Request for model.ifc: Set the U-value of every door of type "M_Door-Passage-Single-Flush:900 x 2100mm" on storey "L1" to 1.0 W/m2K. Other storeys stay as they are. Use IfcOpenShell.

First a look at what the model holds.

```python
import ifcopenshell
import ifcopenshell.util.element

model = ifcopenshell.open("model.ifc")
print(model.schema)
storey = next(s for s in model.by_type("IfcBuildingStorey") if s.Name == "L1")
doors = [e for e in ifcopenshell.util.element.get_decomposition(storey) if e.is_a("IfcDoor")]
seen = {}
for e in doors:
    element_type = ifcopenshell.util.element.get_type(e)
    key = (element_type.Name if element_type != e and element_type else None, ifcopenshell.util.element.get_pset(e, "Pset_DoorCommon", "ThermalTransmittance"))
    seen[key] = seen.get(key, 0) + 1
for (name, value), count in sorted(seen.items(), key=str):
    print(count, "x", name, "|", value)
```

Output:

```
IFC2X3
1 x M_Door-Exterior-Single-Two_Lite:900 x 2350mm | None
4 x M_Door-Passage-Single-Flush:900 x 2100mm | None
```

```python
import ifcopenshell
import ifcopenshell.api.pset
import ifcopenshell.util.element

model = ifcopenshell.open("model.ifc")

storey = next(s for s in model.by_type("IfcBuildingStorey") if s.Name == "L1")
doors = [e for e in ifcopenshell.util.element.get_decomposition(storey) if e.is_a("IfcDoor")]

count = 0
for e in doors:
    element_type = ifcopenshell.util.element.get_type(e)
    if element_type in (None, e) or element_type.Name != "M_Door-Passage-Single-Flush:900 x 2100mm":
        continue
    # add_pset returns the element's existing set when there is one.
    pset = ifcopenshell.api.pset.add_pset(model, product=e, name="Pset_DoorCommon")
    ifcopenshell.api.pset.edit_pset(model, pset=pset, properties={"ThermalTransmittance": 1.0})
    count += 1

print(count, "doors updated")

model.write("model_edited.ifc")
```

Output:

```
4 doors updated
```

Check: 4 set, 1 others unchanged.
